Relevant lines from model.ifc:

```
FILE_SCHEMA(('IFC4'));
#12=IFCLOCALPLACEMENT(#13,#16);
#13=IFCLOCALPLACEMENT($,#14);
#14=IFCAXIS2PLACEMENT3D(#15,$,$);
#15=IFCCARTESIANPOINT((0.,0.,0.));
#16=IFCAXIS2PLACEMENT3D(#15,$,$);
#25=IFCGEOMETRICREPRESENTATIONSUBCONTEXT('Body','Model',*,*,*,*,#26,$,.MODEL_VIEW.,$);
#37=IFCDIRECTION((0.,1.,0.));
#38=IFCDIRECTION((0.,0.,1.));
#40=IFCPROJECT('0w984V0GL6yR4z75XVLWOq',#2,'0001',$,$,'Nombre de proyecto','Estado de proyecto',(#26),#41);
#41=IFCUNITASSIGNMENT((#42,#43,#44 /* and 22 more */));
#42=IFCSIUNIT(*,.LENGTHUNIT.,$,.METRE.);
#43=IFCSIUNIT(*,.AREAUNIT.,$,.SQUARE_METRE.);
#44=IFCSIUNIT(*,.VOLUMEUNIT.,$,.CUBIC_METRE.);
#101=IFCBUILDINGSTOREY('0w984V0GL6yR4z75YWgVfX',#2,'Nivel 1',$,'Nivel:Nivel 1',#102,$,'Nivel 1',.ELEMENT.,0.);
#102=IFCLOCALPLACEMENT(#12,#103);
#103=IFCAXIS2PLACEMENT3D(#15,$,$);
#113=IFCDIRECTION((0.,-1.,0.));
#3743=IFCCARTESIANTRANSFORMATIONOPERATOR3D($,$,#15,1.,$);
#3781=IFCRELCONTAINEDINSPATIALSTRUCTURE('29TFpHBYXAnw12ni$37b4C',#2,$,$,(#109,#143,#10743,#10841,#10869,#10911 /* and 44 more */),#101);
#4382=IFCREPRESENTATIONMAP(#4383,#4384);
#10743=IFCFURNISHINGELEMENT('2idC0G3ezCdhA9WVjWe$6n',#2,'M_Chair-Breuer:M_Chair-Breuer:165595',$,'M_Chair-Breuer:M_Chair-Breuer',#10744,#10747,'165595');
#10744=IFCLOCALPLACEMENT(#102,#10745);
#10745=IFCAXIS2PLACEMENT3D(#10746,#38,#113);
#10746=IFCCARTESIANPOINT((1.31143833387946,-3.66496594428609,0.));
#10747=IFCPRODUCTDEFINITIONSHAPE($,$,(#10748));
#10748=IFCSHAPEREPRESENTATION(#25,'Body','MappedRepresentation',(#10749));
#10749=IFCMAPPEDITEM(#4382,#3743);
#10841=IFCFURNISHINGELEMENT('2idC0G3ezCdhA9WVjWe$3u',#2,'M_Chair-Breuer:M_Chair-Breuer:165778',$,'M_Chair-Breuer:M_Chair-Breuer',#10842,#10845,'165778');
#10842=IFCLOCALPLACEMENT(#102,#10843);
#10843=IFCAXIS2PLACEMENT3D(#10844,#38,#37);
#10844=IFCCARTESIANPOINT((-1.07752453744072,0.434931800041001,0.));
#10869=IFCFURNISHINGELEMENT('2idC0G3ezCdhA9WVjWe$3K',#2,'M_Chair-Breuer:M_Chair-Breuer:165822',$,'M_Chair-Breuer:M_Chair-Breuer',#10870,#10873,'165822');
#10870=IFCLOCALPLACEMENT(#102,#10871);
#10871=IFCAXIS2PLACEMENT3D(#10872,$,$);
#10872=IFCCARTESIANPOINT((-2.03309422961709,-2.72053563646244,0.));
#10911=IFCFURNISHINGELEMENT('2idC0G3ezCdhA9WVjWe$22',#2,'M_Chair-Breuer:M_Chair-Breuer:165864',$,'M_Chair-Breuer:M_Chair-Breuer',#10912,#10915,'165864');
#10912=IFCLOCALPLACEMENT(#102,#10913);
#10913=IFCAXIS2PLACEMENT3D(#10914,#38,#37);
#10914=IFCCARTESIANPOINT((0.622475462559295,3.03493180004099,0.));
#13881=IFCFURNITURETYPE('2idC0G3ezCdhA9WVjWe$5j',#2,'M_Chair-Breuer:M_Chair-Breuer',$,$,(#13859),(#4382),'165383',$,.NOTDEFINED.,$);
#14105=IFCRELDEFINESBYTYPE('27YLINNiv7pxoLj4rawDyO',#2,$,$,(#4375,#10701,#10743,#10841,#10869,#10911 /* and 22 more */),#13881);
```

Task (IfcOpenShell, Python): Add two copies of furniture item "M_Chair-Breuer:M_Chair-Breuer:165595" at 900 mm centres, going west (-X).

```python
import numpy as np
import ifcopenshell
import ifcopenshell.api.geometry
import ifcopenshell.api.root
import ifcopenshell.util.element
import ifcopenshell.util.placement
import ifcopenshell.util.unit

model = ifcopenshell.open("model.ifc")
unit_scale = ifcopenshell.util.unit.calculate_unit_scale(model)


def reuse_history(source, copy):
    """copy_class also copies each property set's owner history, people and application; keep the originals."""
    for rel in copy.IsDefinedBy:
        if rel.is_a("IfcRelDefinesByProperties") and (history := rel.RelatingPropertyDefinition.OwnerHistory):
            rel.RelatingPropertyDefinition.OwnerHistory = source.OwnerHistory
            ifcopenshell.util.element.remove_deep2(model, history)


source = model.by_guid("2idC0G3ezCdhA9WVjWe$6n")
base = ifcopenshell.util.placement.get_local_placement(source.ObjectPlacement)
step = np.array([-1.0, 0.0, 0.0]) * 0.9 / unit_scale

for i in range(1, 3):
    copy = ifcopenshell.api.root.copy_class(model, product=source)
    copy.Representation = ifcopenshell.util.element.copy_deep(
        model, source.Representation, exclude=["IfcGeometricRepresentationContext", "IfcRepresentationMap"]
    )
    copy.Name = "M_Chair-Breuer:M_Chair-Breuer"
    copy.Tag = None
    reuse_history(source, copy)
    matrix = base.copy()
    matrix[:3, 3] += i * step
    print("added at", matrix[:3, 3].round(3) + 0.0)
    ifcopenshell.api.geometry.edit_object_placement(model, product=copy, matrix=matrix, is_si=False)

model.write("model_rev.ifc")
```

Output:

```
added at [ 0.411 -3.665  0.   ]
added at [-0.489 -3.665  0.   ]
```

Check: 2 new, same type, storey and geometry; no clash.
